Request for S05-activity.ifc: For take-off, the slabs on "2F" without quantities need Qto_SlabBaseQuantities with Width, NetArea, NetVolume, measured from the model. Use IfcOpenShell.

First a look at what the model holds.

```python
import ifcopenshell
import ifcopenshell.util.element
import ifcopenshell.util.unit

model = ifcopenshell.open("S05-activity.ifc")
print(model.schema)
for unit_type in ("LENGTHUNIT", "AREAUNIT", "VOLUMEUNIT"):
    print(unit_type, ifcopenshell.util.unit.calculate_unit_scale(model, unit_type))
storey = next(s for s in model.by_type("IfcBuildingStorey") if s.Name == "2F")
slabs = [e for e in ifcopenshell.util.element.get_decomposition(storey) if e.is_a("IfcSlab")]
for e in sorted(slabs, key=lambda e: e.id()):
    print(e.id(), e.is_a(), e.Name, list(ifcopenshell.util.element.get_psets(e, qtos_only=True)), sep=" | ")
```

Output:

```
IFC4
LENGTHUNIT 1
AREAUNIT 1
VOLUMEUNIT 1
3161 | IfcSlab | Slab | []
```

```python
import ifcopenshell
import ifcopenshell.api.pset
import ifcopenshell.geom
import ifcopenshell.util.element
import ifcopenshell.util.shape
import ifcopenshell.util.unit

model = ifcopenshell.open("S05-activity.ifc")
unit_scale = ifcopenshell.util.unit.calculate_unit_scale(model)
area_scale = ifcopenshell.util.unit.calculate_unit_scale(model, "AREAUNIT")
volume_scale = ifcopenshell.util.unit.calculate_unit_scale(model, "VOLUMEUNIT")
settings = ifcopenshell.geom.settings()

storey = next(s for s in model.by_type("IfcBuildingStorey") if s.Name == "2F")
slabs = [e for e in ifcopenshell.util.element.get_decomposition(storey) if e.is_a("IfcSlab")]

for e in sorted(slabs, key=lambda e: e.id()):
    if ifcopenshell.util.element.get_psets(e, qtos_only=True, should_inherit=False):
        continue
    # Geometry comes back in metres, in the element's own axes.
    shape = ifcopenshell.geom.create_shape(settings, e)
    values = {
        "Width": ifcopenshell.util.shape.get_z(shape.geometry) / unit_scale,
        "NetArea": ifcopenshell.util.shape.get_footprint_area(shape.geometry) / area_scale,
        "NetVolume": ifcopenshell.util.shape.get_volume(shape.geometry) / volume_scale,
    }
    qto = ifcopenshell.api.pset.add_qto(model, product=e, name="Qto_SlabBaseQuantities")
    ifcopenshell.api.pset.edit_qto(model, qto=qto, properties=values)
    print(e.id(), {k: round(v, 3) for k, v in values.items()})

model.write("S05-activity_rev.ifc")
```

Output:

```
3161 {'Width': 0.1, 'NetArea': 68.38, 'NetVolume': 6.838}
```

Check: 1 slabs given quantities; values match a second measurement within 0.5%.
